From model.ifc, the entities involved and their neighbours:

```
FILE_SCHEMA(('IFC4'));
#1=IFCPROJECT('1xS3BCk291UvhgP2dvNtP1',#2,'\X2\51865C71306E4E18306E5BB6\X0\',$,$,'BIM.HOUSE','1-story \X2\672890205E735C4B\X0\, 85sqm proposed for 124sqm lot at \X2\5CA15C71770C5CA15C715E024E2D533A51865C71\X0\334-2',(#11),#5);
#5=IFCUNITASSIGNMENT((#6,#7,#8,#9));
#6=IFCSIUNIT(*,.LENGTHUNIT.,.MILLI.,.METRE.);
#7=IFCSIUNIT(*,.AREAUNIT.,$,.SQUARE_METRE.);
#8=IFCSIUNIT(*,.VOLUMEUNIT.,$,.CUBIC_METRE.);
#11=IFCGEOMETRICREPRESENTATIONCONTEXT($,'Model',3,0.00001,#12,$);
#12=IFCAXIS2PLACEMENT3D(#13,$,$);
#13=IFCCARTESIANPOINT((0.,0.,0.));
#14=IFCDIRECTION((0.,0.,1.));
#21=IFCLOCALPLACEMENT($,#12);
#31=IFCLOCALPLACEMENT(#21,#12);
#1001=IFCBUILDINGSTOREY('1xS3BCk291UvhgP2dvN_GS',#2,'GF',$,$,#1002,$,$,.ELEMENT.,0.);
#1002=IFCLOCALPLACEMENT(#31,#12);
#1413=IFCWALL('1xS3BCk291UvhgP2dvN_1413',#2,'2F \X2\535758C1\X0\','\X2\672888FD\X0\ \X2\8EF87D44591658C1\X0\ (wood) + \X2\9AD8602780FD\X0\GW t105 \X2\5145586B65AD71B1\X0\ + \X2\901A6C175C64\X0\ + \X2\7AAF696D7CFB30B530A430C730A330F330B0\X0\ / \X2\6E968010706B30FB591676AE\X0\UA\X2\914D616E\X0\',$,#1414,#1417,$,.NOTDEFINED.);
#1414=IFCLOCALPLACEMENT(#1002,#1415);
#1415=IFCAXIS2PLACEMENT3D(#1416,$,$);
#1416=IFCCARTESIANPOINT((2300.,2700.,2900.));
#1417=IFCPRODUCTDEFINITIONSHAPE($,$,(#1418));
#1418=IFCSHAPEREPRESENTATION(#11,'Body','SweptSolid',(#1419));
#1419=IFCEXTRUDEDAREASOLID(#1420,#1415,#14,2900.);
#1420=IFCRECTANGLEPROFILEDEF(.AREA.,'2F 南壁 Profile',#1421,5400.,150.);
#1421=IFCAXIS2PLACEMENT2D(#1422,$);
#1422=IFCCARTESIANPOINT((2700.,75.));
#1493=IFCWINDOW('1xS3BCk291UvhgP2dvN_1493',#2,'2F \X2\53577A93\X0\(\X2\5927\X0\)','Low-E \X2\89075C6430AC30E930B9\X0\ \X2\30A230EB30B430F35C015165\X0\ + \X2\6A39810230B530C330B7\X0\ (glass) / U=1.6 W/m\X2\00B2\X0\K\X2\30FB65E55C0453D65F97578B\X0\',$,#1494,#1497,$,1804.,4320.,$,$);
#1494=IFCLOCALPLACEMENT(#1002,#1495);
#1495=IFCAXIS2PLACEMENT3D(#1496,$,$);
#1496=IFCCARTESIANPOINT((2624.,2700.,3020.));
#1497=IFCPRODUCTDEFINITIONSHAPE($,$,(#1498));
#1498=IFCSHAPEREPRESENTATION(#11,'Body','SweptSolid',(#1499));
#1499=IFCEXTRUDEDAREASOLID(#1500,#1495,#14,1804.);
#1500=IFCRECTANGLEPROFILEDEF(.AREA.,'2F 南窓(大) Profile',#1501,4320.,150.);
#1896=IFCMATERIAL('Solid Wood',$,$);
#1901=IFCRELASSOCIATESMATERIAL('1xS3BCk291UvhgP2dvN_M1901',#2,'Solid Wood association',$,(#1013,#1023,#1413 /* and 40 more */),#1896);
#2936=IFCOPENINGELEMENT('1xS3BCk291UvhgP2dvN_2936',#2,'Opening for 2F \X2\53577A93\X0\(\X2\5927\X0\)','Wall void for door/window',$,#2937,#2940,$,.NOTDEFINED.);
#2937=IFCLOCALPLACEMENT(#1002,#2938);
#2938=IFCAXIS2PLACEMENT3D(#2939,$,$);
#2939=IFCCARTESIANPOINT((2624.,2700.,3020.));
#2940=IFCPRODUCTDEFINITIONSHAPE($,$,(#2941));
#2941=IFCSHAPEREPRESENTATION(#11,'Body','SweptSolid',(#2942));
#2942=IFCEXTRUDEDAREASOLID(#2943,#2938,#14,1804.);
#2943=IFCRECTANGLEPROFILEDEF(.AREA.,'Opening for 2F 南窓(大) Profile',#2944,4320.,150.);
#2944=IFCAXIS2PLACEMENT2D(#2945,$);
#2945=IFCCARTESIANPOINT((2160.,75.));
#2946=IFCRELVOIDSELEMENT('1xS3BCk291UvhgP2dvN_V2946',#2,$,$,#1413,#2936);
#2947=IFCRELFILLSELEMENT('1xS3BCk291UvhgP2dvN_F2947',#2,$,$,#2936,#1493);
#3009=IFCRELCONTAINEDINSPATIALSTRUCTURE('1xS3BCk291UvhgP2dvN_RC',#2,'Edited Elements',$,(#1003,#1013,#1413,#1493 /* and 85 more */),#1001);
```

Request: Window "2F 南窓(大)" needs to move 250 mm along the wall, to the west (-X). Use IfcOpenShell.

```python
import ifcopenshell
import ifcopenshell.api.geometry
import ifcopenshell.util.placement

model = ifcopenshell.open("model.ifc")

window = model.by_id(1493)
opening = window.FillsVoids[0].RelatingOpeningElement
wall = opening.VoidsElements[0].RelatingBuildingElement

wall_matrix = ifcopenshell.util.placement.get_local_placement(wall.ObjectPlacement)
shift = wall_matrix[:3, 0] * -250.0
before = ifcopenshell.util.placement.get_local_placement(window.ObjectPlacement)[:3, 3].copy()

# The window is not placed relative to its opening, so move both.
for product in (opening, window):
    matrix = ifcopenshell.util.placement.get_local_placement(product.ObjectPlacement)
    matrix[:3, 3] += shift
    ifcopenshell.api.geometry.edit_object_placement(model, product=product, matrix=matrix, is_si=False)

after = ifcopenshell.util.placement.get_local_placement(window.ObjectPlacement)[:3, 3]
print("window moved by", (after - before).round(3) + 0.0)

model.write("model_rev.ifc")
```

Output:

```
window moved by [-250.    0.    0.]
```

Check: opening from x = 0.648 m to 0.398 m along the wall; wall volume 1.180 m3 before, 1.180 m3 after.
